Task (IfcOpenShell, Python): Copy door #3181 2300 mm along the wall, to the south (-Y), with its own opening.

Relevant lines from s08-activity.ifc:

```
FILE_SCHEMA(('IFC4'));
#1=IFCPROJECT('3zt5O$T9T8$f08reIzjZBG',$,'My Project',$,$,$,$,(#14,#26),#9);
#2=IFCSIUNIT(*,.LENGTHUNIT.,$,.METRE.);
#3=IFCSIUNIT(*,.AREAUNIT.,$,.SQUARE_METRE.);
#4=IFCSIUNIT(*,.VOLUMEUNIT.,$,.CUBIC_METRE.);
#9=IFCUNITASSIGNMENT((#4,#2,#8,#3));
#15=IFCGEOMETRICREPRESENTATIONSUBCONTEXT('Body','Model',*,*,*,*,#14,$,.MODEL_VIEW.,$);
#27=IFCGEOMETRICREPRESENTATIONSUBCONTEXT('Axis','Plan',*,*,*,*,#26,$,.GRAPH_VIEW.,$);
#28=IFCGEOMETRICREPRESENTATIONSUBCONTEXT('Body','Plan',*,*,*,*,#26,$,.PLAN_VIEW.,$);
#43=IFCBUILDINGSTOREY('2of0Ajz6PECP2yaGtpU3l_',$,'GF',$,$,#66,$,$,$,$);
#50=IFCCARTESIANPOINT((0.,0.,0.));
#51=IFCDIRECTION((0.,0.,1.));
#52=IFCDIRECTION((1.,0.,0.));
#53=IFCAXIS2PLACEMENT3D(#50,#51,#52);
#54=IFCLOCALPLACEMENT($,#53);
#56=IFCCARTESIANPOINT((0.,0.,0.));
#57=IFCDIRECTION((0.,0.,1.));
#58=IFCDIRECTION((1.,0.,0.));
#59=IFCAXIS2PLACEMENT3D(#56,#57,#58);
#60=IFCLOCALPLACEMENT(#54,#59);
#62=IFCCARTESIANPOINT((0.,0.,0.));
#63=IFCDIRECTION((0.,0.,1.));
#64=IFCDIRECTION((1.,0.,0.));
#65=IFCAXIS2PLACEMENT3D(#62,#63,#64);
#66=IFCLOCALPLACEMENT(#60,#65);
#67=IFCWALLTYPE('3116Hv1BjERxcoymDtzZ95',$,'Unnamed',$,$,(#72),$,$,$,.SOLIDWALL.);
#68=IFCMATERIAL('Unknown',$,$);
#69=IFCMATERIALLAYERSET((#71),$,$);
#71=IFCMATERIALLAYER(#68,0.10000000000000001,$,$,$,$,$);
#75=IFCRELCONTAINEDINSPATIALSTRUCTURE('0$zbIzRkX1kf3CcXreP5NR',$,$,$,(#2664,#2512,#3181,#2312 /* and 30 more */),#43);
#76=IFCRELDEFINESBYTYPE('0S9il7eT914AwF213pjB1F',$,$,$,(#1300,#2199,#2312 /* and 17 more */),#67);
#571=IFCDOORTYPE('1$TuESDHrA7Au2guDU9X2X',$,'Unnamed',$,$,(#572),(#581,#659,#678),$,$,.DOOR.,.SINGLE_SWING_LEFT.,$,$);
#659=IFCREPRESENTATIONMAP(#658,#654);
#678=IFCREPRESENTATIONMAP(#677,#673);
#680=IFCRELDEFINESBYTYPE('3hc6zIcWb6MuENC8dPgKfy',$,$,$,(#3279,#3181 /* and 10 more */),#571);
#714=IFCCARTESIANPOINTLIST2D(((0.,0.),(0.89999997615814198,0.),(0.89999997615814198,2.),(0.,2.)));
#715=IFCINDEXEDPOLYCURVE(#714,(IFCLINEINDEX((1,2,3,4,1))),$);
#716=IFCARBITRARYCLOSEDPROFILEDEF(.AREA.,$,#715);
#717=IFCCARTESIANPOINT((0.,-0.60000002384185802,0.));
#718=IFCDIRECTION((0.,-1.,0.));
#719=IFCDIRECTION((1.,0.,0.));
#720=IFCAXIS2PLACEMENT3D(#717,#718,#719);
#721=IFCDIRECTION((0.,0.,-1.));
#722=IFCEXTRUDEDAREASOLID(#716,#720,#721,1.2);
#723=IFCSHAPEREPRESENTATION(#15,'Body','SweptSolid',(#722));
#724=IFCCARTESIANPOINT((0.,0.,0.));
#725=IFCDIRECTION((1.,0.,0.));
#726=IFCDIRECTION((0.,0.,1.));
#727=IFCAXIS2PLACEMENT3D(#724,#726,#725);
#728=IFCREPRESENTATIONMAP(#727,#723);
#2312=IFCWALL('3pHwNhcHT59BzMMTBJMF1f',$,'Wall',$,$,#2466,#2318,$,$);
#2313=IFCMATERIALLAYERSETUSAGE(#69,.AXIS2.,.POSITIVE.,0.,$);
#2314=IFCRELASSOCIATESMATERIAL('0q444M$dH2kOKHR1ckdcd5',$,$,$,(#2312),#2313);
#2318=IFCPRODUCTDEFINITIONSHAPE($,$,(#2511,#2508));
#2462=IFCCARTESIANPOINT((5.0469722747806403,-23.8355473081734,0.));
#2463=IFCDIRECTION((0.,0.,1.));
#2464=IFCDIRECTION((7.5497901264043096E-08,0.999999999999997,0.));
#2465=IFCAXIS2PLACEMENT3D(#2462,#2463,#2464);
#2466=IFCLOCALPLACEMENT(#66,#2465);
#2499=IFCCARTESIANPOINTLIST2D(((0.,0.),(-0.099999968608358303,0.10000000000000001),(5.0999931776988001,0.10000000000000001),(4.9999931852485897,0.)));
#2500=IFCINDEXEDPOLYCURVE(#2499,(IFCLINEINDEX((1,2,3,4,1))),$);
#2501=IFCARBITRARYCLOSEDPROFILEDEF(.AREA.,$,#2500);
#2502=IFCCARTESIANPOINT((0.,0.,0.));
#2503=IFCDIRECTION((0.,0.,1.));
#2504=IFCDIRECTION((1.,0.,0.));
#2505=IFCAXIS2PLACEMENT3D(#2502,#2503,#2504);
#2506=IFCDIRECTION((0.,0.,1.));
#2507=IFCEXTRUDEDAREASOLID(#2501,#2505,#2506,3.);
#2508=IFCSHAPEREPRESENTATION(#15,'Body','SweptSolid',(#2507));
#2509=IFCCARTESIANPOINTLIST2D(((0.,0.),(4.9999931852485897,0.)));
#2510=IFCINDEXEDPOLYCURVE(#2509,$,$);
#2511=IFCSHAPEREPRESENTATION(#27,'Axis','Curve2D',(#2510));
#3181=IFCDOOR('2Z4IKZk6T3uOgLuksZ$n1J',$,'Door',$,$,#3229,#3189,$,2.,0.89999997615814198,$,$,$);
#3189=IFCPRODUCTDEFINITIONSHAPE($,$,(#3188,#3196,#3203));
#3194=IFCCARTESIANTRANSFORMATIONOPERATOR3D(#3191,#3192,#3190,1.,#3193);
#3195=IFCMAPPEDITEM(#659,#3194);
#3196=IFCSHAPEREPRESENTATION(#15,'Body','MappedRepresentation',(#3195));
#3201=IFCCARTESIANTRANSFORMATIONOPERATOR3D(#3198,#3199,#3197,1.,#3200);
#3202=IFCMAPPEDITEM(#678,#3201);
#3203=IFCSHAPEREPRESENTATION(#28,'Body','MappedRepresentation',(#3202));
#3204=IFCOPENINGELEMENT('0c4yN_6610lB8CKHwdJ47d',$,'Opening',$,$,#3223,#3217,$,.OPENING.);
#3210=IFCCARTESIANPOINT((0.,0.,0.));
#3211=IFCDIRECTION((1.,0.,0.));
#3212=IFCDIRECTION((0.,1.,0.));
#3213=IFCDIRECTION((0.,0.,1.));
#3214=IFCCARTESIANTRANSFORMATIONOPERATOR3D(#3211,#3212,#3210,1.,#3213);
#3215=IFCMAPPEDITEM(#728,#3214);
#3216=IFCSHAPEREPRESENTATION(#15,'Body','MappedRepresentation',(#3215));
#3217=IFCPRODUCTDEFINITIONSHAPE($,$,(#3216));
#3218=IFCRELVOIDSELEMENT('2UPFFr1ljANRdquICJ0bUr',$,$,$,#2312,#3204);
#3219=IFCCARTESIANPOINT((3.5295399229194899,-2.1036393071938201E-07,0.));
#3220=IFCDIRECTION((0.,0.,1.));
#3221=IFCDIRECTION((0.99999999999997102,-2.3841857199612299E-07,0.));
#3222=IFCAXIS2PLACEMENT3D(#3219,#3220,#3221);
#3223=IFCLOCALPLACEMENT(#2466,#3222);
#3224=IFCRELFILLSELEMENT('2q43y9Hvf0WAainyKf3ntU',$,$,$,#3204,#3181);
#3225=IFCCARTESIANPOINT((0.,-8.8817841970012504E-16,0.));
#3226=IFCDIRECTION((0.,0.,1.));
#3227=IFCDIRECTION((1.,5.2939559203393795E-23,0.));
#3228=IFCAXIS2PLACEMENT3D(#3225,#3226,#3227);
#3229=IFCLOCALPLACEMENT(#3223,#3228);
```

```python
import ifcopenshell
import ifcopenshell.api.feature
import ifcopenshell.api.geometry
import ifcopenshell.api.root
import ifcopenshell.geom
import ifcopenshell.util.element
import ifcopenshell.util.placement
import ifcopenshell.util.shape
import ifcopenshell.util.unit

model = ifcopenshell.open("s08-activity.ifc")
unit_scale = ifcopenshell.util.unit.calculate_unit_scale(model)
settings = ifcopenshell.geom.settings()


def volume(element):
    """Net volume in cubic metres, openings subtracted."""
    shape = ifcopenshell.geom.create_shape(settings, element)
    return ifcopenshell.util.shape.get_volume(shape.geometry)


door = model.by_id(3181)
opening = door.FillsVoids[0].RelatingOpeningElement
wall = opening.VoidsElements[0].RelatingBuildingElement
before = volume(wall)
shift = ifcopenshell.util.placement.get_local_placement(wall.ObjectPlacement)[:3, 0] * -2.3 / unit_scale

# copy_class copies the void relationship, type, container and properties, but no geometry.
new_opening = ifcopenshell.api.root.copy_class(model, product=opening)
new_opening.Representation = ifcopenshell.util.element.copy_deep(
    model, opening.Representation, exclude=["IfcGeometricRepresentationContext", "IfcRepresentationMap"]
)
new_door = ifcopenshell.api.root.copy_class(model, product=door)
new_door.Representation = ifcopenshell.util.element.copy_deep(
    model, door.Representation, exclude=["IfcGeometricRepresentationContext", "IfcRepresentationMap"]
)
ifcopenshell.api.feature.add_filling(model, opening=new_opening, element=new_door)

for old, new in ((opening, new_opening), (door, new_door)):
    matrix = ifcopenshell.util.placement.get_local_placement(old.ObjectPlacement)
    matrix[:3, 3] += shift
    ifcopenshell.api.geometry.edit_object_placement(model, product=new, matrix=matrix, is_si=False)

after = volume(wall)

print(f"wall volume {before:.3f} -> {after:.3f} m3")

model.write("s08-activity_v2.ifc")
```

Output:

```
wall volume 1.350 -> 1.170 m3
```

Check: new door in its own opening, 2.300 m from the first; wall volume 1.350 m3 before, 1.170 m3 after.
